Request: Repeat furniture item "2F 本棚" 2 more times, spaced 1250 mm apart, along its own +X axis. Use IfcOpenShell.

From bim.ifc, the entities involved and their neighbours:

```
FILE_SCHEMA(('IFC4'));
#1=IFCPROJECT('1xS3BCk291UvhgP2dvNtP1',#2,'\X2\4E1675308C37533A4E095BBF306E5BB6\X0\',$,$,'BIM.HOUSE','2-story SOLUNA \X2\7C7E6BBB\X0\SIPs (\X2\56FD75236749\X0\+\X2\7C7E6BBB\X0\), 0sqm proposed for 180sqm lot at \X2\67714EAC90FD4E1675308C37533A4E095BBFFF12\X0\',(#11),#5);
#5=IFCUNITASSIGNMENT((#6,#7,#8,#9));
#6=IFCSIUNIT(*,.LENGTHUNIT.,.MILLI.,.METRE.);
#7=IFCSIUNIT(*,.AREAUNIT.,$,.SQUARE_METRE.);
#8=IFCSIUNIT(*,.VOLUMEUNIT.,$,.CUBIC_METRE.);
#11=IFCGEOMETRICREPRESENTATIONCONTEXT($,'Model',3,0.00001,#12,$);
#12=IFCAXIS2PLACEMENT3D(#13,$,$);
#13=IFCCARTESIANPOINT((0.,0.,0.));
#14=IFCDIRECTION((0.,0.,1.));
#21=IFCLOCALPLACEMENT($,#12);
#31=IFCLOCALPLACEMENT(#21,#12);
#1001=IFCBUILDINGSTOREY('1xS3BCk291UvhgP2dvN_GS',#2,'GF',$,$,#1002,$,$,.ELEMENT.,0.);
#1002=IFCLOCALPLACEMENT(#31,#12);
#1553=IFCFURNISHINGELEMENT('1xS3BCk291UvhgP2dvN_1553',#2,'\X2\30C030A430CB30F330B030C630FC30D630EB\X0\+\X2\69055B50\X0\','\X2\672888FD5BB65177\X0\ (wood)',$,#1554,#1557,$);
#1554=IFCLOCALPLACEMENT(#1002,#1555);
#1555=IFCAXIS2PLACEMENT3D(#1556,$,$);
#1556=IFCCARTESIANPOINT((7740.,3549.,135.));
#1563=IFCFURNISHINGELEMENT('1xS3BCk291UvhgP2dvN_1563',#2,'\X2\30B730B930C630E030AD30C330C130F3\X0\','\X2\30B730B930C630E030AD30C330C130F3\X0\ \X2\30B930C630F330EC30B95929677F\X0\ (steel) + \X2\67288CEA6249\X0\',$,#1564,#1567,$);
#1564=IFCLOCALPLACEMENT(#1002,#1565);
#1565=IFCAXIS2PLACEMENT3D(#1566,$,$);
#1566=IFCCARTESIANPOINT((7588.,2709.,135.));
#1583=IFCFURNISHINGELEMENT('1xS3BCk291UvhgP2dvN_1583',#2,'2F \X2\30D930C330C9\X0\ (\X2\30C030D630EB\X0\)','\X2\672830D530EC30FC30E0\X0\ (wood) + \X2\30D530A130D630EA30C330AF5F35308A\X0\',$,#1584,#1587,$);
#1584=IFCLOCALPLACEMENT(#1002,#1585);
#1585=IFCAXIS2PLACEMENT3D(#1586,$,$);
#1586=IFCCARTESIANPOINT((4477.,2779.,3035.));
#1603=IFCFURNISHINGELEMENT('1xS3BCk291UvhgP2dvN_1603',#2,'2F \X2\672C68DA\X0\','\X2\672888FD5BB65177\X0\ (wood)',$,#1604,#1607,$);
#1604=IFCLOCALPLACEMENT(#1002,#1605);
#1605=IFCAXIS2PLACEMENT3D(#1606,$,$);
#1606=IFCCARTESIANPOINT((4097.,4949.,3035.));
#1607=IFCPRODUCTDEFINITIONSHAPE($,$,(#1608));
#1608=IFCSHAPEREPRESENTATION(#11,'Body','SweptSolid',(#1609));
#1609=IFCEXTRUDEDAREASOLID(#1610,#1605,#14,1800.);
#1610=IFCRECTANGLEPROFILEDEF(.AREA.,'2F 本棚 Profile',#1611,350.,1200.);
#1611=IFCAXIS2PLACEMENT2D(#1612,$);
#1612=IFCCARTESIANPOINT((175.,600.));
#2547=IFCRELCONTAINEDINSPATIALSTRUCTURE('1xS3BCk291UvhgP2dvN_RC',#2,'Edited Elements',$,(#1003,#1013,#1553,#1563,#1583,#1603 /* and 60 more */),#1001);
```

```python
import ifcopenshell
import ifcopenshell.api.geometry
import ifcopenshell.api.root
import ifcopenshell.util.element
import ifcopenshell.util.placement

model = ifcopenshell.open("bim.ifc")


def reuse_history(source, copy):
    """copy_class also copies each property set's owner history, people and application; keep the originals."""
    for rel in copy.IsDefinedBy:
        if rel.is_a("IfcRelDefinesByProperties") and (history := rel.RelatingPropertyDefinition.OwnerHistory):
            rel.RelatingPropertyDefinition.OwnerHistory = source.OwnerHistory
            ifcopenshell.util.element.remove_deep2(model, history)


source = model.by_guid("1xS3BCk291UvhgP2dvN_1603")
base = ifcopenshell.util.placement.get_local_placement(source.ObjectPlacement)
step = base[:3, 0] * 1250.0

for i in range(1, 3):
    copy = ifcopenshell.api.root.copy_class(model, product=source)
    copy.Representation = ifcopenshell.util.element.copy_deep(
        model, source.Representation, exclude=["IfcGeometricRepresentationContext", "IfcRepresentationMap"]
    )
    reuse_history(source, copy)
    matrix = base.copy()
    matrix[:3, 3] += i * step
    print("added at", matrix[:3, 3].round(3) + 0.0)
    ifcopenshell.api.geometry.edit_object_placement(model, product=copy, matrix=matrix, is_si=False)

model.write("bim-out.ifc")
```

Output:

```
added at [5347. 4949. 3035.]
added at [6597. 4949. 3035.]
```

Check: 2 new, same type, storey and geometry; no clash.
